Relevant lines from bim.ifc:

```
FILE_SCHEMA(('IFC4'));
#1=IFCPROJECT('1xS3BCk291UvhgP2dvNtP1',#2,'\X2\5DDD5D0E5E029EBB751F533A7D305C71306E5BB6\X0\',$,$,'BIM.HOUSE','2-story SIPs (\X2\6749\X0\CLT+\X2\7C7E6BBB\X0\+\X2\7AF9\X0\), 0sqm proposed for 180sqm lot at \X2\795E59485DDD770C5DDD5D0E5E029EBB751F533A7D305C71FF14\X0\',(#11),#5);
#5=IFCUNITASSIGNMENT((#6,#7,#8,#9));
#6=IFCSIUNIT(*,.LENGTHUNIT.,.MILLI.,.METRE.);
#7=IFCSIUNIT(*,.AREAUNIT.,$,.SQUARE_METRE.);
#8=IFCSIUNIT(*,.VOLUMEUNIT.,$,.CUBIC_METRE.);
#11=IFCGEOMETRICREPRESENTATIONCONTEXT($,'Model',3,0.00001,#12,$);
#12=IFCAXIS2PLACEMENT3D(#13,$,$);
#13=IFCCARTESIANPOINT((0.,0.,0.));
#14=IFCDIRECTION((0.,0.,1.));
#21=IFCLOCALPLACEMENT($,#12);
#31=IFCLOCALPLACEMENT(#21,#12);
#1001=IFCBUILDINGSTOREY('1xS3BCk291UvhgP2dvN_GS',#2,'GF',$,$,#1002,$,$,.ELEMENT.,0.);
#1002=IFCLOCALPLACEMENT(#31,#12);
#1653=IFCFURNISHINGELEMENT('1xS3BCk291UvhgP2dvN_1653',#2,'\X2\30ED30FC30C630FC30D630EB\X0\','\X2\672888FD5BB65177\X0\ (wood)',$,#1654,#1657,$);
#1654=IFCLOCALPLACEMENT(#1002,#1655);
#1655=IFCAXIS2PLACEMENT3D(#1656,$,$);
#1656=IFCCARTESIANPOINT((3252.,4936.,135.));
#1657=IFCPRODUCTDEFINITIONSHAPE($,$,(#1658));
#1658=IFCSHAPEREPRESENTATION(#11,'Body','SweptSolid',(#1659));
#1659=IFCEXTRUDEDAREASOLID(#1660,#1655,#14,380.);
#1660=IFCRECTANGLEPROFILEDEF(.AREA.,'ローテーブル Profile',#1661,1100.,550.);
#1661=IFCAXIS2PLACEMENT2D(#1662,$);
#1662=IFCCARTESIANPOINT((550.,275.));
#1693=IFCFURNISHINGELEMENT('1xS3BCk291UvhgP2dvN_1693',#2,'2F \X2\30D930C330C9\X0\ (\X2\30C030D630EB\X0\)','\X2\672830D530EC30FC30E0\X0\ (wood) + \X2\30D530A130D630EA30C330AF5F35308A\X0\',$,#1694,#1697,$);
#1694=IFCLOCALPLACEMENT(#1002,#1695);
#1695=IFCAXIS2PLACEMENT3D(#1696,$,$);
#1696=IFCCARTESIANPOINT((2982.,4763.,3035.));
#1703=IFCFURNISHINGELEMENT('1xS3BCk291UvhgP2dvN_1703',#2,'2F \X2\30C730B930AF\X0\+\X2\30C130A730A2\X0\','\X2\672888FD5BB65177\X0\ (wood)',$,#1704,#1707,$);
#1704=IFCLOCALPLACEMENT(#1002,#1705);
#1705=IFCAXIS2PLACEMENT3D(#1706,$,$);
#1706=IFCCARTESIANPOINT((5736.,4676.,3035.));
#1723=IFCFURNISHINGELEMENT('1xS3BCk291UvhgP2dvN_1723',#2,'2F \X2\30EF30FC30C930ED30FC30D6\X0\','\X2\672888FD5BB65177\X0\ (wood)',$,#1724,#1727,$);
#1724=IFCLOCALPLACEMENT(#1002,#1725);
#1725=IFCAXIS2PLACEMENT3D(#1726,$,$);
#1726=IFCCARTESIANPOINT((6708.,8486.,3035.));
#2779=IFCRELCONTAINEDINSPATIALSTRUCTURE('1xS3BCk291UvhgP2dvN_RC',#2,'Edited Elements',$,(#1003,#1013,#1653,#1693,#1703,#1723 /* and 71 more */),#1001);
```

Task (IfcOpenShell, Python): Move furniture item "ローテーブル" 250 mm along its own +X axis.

```python
import ifcopenshell
import ifcopenshell.api.geometry
import ifcopenshell.util.placement
import ifcopenshell.util.unit

model = ifcopenshell.open("bim.ifc")
unit_scale = ifcopenshell.util.unit.calculate_unit_scale(model)

item = model.by_id(1653)
matrix = ifcopenshell.util.placement.get_local_placement(item.ObjectPlacement)
matrix[:3, 3] += matrix[:3, 0] * 0.25 / unit_scale
ifcopenshell.api.geometry.edit_object_placement(model, product=item, matrix=matrix, is_si=False)

print(ifcopenshell.util.placement.get_local_placement(item.ObjectPlacement).round(3) + 0.0)

model.write("bim_rev.ifc")
```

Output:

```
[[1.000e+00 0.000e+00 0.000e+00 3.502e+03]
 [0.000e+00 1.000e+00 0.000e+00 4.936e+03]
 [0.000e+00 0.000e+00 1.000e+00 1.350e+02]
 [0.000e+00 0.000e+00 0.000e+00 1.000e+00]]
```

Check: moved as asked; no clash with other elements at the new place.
